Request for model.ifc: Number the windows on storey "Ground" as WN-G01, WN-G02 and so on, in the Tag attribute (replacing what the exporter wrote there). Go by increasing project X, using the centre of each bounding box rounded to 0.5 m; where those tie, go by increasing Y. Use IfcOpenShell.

First a look at what the model holds.

```python
import ifcopenshell
import ifcopenshell.util.element
import ifcopenshell.util.placement

model = ifcopenshell.open("model.ifc")
print(model.schema)
storey = next(s for s in model.by_type("IfcBuildingStorey") if s.Name == "Ground")
windows = [e for e in ifcopenshell.util.element.get_decomposition(storey) if e.is_a("IfcWindow")]
for e in sorted(windows, key=lambda e: e.id()):
    origin = ifcopenshell.util.placement.get_local_placement(e.ObjectPlacement)[:3, 3]
    print(e.id(), e.Tag, e.Name, origin.round(2) + 0.0, sep=" | ")
```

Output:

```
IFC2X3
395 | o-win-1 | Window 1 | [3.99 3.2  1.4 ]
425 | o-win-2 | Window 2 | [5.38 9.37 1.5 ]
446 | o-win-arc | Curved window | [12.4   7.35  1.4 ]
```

```python
import ifcopenshell
import ifcopenshell.geom
import ifcopenshell.util.element
import ifcopenshell.util.shape

model = ifcopenshell.open("model.ifc")
settings = ifcopenshell.geom.settings()
settings.set("use-world-coords", True)


def centre(element):
    shape = ifcopenshell.geom.create_shape(settings, element)
    return ifcopenshell.util.shape.get_bbox_centroid(shape.geometry)


storey = next(s for s in model.by_type("IfcBuildingStorey") if s.Name == "Ground")
windows = [e for e in ifcopenshell.util.element.get_decomposition(storey) if e.is_a("IfcWindow")]

# Insertion points can sit at a corner or the storey origin, so sort by the geometry (in metres).
centres = {e: centre(e) for e in windows}
windows.sort(key=lambda e: (round(centres[e][0] / 0.5), centres[e][1]))

for i, e in enumerate(windows, start=1):
    number = f"WN-G{i:02d}"
    e.Tag = number
    print(e.id(), number)

model.write("model-out.ifc")
```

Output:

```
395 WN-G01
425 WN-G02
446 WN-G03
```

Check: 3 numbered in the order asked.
